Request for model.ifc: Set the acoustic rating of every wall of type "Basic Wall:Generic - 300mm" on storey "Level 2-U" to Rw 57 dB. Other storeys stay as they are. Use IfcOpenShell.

First a look at what the model holds.

```python
import ifcopenshell
import ifcopenshell.util.element

model = ifcopenshell.open("model.ifc")
print(model.schema)
storey = next(s for s in model.by_type("IfcBuildingStorey") if s.Name == "Level 2-U")
walls = [e for e in ifcopenshell.util.element.get_decomposition(storey) if e.is_a("IfcWall")]
seen = {}
for e in walls:
    element_type = ifcopenshell.util.element.get_type(e)
    key = (element_type.Name if element_type != e and element_type else None, ifcopenshell.util.element.get_pset(e, "Pset_WallCommon", "AcousticRating"))
    seen[key] = seen.get(key, 0) + 1
for (name, value), count in sorted(seen.items(), key=str):
    print(count, "x", name, "|", value)
```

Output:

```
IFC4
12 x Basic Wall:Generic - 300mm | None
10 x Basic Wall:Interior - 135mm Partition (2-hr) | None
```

```python
import ifcopenshell
import ifcopenshell.api.pset
import ifcopenshell.util.element

model = ifcopenshell.open("model.ifc")

storey = next(s for s in model.by_type("IfcBuildingStorey") if s.Name == "Level 2-U")
walls = [e for e in ifcopenshell.util.element.get_decomposition(storey) if e.is_a("IfcWall")]

count = 0
for e in walls:
    element_type = ifcopenshell.util.element.get_type(e)
    if element_type in (None, e) or element_type.Name != "Basic Wall:Generic - 300mm":
        continue
    # add_pset returns the element's existing set when there is one.
    pset = ifcopenshell.api.pset.add_pset(model, product=e, name="Pset_WallCommon")
    ifcopenshell.api.pset.edit_pset(model, pset=pset, properties={"AcousticRating": "Rw 57 dB"})
    count += 1

print(count, "walls updated")

model.write("model-out.ifc")
```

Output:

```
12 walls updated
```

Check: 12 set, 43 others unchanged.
